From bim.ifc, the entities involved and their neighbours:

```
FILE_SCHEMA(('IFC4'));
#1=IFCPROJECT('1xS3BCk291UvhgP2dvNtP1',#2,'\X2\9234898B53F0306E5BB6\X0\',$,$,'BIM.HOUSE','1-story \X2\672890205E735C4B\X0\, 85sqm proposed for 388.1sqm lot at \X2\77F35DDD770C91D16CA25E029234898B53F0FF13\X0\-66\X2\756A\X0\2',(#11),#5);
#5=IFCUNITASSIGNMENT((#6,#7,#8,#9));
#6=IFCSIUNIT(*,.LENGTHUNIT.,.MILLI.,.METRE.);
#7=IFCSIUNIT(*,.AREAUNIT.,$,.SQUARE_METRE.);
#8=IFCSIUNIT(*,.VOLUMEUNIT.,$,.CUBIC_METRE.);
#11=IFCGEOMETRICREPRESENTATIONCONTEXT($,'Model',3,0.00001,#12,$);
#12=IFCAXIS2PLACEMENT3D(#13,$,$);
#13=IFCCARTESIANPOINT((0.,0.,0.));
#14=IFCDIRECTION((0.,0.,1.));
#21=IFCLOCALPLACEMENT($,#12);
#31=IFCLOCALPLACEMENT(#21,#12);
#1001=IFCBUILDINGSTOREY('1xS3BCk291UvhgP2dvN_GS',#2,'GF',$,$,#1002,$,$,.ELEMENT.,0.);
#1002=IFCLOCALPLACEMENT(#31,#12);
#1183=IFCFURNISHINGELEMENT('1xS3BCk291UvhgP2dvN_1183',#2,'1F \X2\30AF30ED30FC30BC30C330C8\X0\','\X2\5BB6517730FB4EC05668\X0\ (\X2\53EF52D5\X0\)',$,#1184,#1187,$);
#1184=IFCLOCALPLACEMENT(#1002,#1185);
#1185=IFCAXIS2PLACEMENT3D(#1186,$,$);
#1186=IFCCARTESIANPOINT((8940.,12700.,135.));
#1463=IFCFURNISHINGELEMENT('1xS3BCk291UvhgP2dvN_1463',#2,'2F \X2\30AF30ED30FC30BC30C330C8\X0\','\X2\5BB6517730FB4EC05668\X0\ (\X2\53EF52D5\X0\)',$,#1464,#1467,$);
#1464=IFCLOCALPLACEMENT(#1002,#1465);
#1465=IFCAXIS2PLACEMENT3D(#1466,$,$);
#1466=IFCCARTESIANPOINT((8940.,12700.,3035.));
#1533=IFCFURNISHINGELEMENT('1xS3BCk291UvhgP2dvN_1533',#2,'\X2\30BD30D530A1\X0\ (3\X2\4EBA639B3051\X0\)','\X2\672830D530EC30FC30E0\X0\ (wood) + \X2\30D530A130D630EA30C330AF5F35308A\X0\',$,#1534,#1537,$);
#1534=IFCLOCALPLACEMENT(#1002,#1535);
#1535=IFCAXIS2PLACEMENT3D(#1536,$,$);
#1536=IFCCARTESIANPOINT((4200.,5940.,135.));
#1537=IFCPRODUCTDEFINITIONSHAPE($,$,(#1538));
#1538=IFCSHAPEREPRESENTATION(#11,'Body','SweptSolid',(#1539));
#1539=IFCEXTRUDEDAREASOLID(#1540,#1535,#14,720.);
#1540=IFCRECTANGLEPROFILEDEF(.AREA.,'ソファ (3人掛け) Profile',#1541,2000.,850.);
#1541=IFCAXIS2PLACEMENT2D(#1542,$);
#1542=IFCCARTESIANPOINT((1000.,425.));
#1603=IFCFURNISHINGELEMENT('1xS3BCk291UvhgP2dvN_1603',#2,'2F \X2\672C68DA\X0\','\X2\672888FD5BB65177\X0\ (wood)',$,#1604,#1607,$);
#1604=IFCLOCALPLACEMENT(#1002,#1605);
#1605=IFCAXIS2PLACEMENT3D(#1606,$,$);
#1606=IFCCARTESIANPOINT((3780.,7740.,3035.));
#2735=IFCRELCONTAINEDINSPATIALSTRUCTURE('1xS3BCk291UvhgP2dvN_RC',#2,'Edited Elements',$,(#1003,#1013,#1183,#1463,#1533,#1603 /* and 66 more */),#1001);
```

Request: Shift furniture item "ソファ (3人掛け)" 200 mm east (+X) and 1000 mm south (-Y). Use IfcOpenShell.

```python
import ifcopenshell
import ifcopenshell.api.geometry
import ifcopenshell.util.placement
import ifcopenshell.util.unit

model = ifcopenshell.open("bim.ifc")
unit_scale = ifcopenshell.util.unit.calculate_unit_scale(model)

item = model.by_guid("1xS3BCk291UvhgP2dvN_1533")
matrix = ifcopenshell.util.placement.get_local_placement(item.ObjectPlacement)
matrix[0, 3] += 0.2 / unit_scale
matrix[1, 3] -= 1 / unit_scale
ifcopenshell.api.geometry.edit_object_placement(model, product=item, matrix=matrix, is_si=False)

print(ifcopenshell.util.placement.get_local_placement(item.ObjectPlacement).round(3) + 0.0)

model.write("bim_rev.ifc")
```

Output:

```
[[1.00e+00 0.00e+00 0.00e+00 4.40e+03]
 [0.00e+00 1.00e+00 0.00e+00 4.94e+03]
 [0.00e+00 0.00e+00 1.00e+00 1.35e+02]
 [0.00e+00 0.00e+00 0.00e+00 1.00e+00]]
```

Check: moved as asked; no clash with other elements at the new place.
